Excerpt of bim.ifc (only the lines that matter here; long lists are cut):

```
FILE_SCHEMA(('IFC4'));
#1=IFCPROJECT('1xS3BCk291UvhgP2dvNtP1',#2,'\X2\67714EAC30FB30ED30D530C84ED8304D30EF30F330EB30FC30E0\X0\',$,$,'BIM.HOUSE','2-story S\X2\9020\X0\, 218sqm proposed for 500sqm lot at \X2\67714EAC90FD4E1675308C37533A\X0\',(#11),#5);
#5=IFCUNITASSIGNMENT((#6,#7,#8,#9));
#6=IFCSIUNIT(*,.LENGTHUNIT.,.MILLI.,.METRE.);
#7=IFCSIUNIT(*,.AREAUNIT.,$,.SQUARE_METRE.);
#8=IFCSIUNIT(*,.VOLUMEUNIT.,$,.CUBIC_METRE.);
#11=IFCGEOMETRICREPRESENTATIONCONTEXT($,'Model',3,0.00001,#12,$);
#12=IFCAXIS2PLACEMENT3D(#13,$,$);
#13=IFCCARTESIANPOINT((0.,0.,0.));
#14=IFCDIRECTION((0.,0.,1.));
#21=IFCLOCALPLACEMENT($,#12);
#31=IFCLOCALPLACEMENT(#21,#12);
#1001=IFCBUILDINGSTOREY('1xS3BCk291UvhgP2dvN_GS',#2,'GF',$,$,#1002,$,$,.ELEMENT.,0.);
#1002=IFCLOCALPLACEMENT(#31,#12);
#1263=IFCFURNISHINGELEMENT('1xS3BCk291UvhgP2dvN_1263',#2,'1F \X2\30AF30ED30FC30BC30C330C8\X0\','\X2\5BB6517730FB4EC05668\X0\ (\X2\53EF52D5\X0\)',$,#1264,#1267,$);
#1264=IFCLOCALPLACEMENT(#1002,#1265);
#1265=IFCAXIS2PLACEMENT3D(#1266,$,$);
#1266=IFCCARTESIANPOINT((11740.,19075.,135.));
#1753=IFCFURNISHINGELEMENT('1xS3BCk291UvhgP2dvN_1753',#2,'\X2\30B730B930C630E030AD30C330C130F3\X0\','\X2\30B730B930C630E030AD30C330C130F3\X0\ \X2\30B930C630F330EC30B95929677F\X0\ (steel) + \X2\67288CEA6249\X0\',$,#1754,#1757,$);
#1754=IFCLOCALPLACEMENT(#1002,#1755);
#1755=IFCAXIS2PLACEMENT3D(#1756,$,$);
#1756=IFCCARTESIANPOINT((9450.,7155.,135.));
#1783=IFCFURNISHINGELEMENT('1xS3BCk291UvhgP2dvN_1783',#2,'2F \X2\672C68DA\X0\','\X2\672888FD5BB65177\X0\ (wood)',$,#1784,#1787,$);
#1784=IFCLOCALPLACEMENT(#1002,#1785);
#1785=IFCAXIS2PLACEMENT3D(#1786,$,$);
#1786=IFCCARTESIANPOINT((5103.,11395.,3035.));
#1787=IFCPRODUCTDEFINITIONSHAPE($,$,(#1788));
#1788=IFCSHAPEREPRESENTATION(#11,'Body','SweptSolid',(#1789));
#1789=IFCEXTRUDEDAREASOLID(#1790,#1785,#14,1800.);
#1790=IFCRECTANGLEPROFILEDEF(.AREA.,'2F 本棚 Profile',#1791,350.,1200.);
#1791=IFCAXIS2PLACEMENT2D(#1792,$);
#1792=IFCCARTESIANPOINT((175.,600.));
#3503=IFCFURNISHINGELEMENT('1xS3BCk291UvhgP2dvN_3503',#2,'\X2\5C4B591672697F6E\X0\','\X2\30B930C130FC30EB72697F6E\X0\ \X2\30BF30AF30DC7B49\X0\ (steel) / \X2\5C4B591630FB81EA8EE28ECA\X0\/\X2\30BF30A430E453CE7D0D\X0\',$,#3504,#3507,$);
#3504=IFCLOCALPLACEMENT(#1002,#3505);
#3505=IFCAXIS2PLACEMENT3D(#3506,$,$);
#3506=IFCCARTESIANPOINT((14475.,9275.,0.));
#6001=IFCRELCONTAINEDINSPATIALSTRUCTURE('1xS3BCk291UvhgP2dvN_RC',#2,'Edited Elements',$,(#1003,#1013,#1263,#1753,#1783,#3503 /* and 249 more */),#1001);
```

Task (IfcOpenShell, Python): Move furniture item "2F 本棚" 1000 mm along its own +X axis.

```python
import ifcopenshell
import ifcopenshell.api.geometry
import ifcopenshell.util.placement
import ifcopenshell.util.unit

model = ifcopenshell.open("bim.ifc")
unit_scale = ifcopenshell.util.unit.calculate_unit_scale(model)

item = model.by_guid("1xS3BCk291UvhgP2dvN_1783")
matrix = ifcopenshell.util.placement.get_local_placement(item.ObjectPlacement)
matrix[:3, 3] += matrix[:3, 0] * 1 / unit_scale
ifcopenshell.api.geometry.edit_object_placement(model, product=item, matrix=matrix, is_si=False)

print(ifcopenshell.util.placement.get_local_placement(item.ObjectPlacement).round(3) + 0.0)

model.write("bim-out.ifc")
```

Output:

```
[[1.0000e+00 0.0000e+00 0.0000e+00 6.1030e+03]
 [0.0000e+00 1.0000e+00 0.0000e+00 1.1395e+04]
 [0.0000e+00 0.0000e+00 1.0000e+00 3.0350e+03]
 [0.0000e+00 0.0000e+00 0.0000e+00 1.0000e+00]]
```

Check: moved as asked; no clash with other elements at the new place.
